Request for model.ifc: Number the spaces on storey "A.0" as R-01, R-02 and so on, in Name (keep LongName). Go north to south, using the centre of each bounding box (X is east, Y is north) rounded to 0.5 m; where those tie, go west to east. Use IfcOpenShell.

First a look at what the model holds.

```python
import ifcopenshell
import ifcopenshell.util.element
import ifcopenshell.util.placement

model = ifcopenshell.open("model.ifc")
print(model.schema)
storey = next(s for s in model.by_type("IfcBuildingStorey") if s.Name == "A.0")
spaces = [e for e in ifcopenshell.util.element.get_decomposition(storey) if e.is_a("IfcSpace")]
for e in sorted(spaces, key=lambda e: e.id()):
    origin = ifcopenshell.util.placement.get_local_placement(e.ObjectPlacement)[:3, 3]
    print(e.id(), e.Name, e.LongName, origin.round(2) + 0.0, sep=" | ")
```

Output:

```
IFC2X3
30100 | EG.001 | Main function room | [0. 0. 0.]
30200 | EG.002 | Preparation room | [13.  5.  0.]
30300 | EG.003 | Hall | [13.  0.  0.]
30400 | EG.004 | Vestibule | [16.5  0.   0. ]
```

```python
import ifcopenshell
import ifcopenshell.geom
import ifcopenshell.util.element
import ifcopenshell.util.shape

model = ifcopenshell.open("model.ifc")
settings = ifcopenshell.geom.settings()
settings.set("use-world-coords", True)


def centre(element):
    shape = ifcopenshell.geom.create_shape(settings, element)
    return ifcopenshell.util.shape.get_bbox_centroid(shape.geometry)


storey = next(s for s in model.by_type("IfcBuildingStorey") if s.Name == "A.0")
spaces = [e for e in ifcopenshell.util.element.get_decomposition(storey) if e.is_a("IfcSpace")]

# Insertion points can sit at a corner or the storey origin, so sort by the geometry (in metres).
centres = {e: centre(e) for e in spaces}
spaces.sort(key=lambda e: (-round(centres[e][1] / 0.5), centres[e][0]))

for i, e in enumerate(spaces, start=1):
    number = f"R-{i:02d}"
    e.Name = number
    print(e.id(), number)

model.write("model_edited.ifc")
```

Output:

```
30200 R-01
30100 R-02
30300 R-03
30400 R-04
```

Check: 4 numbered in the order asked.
